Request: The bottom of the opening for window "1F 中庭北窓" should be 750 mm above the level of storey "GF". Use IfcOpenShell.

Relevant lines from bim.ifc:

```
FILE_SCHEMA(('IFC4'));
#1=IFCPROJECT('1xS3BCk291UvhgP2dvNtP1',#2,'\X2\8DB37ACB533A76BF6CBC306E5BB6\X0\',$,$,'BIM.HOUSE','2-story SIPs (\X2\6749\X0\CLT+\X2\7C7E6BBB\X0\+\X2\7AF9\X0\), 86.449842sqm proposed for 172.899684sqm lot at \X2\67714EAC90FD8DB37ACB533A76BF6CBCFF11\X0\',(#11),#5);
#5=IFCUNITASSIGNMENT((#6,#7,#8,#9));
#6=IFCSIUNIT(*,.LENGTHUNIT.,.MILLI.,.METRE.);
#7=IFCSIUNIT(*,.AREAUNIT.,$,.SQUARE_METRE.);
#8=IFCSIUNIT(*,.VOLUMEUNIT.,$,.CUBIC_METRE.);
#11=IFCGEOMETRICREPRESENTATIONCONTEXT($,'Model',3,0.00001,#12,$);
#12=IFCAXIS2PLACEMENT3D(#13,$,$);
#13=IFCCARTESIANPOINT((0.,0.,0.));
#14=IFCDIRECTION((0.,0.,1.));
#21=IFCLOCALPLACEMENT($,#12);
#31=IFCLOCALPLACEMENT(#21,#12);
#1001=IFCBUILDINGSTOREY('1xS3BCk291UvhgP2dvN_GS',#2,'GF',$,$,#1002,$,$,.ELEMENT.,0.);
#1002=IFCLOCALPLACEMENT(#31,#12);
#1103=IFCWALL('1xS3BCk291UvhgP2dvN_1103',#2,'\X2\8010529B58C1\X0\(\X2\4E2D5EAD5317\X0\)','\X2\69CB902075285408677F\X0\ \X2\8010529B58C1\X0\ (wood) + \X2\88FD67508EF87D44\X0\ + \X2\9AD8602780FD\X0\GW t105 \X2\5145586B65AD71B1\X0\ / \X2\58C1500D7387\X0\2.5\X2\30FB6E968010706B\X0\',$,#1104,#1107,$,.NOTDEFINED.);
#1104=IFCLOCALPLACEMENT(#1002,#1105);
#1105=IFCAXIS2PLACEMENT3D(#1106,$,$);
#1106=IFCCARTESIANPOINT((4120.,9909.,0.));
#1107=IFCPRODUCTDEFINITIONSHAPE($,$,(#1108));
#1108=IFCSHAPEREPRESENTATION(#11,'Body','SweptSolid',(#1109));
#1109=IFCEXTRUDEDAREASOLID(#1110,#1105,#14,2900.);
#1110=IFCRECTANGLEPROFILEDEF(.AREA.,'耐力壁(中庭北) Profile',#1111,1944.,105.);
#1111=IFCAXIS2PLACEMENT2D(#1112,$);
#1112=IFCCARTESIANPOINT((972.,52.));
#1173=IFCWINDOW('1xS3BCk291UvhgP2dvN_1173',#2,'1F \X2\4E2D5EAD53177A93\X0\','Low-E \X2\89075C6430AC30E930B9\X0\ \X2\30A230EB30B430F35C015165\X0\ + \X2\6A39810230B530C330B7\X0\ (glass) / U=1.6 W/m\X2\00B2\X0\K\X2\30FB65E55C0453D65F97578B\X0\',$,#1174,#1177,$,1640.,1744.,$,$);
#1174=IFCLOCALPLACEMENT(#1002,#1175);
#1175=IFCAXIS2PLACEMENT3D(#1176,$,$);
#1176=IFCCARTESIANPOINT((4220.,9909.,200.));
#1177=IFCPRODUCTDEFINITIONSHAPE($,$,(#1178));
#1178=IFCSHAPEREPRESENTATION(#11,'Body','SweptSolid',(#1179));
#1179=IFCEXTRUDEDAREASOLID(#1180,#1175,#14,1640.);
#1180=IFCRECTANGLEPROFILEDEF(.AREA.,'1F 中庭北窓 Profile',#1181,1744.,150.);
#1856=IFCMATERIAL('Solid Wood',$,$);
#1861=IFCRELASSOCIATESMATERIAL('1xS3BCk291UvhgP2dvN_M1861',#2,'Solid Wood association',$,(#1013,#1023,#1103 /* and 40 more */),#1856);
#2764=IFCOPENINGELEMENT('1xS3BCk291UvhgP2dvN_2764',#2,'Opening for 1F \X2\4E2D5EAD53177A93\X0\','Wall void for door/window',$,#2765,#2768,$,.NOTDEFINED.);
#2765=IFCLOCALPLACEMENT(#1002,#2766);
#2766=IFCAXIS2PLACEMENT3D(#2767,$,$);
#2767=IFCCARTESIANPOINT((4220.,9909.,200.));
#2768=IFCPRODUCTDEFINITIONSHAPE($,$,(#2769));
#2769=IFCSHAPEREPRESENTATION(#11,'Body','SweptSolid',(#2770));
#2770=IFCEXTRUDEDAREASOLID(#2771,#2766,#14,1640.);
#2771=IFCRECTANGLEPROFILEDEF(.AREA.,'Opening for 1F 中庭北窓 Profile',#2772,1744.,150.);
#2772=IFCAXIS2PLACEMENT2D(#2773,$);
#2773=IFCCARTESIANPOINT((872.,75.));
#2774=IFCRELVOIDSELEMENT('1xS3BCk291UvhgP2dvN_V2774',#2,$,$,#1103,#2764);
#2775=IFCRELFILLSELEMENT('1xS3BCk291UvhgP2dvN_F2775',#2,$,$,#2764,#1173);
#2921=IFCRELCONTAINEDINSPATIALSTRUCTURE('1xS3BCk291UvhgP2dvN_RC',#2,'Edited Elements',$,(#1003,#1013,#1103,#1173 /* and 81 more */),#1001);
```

```python
import numpy as np
import ifcopenshell
import ifcopenshell.api.geometry
import ifcopenshell.geom
import ifcopenshell.util.element
import ifcopenshell.util.placement
import ifcopenshell.util.shape
import ifcopenshell.util.unit

model = ifcopenshell.open("bim.ifc")
unit_scale = ifcopenshell.util.unit.calculate_unit_scale(model)

window = model.by_guid("1xS3BCk291UvhgP2dvN_1173")
opening = window.FillsVoids[0].RelatingOpeningElement
storey = ifcopenshell.util.element.get_container(window, ifc_class="IfcBuildingStorey")
level = ifcopenshell.util.placement.get_local_placement(storey.ObjectPlacement)[2, 3]

# The opening's origin need not be at the sill, so measure its lowest point.
shape = ifcopenshell.geom.create_shape(ifcopenshell.geom.settings(), opening)
bottom = ifcopenshell.util.shape.get_shape_bottom_elevation(shape, shape.geometry) / unit_scale
dz = level + 0.75 / unit_scale - bottom

shift = np.array([0.0, 0.0, dz])
# The window is not placed relative to its opening, so move both.
for product in (opening, window):
    matrix = ifcopenshell.util.placement.get_local_placement(product.ObjectPlacement)
    matrix[:3, 3] += shift
    ifcopenshell.api.geometry.edit_object_placement(model, product=product, matrix=matrix, is_si=False)

print(f"moved by {dz * unit_scale:+.3f} m")

model.write("bim_rev.ifc")
```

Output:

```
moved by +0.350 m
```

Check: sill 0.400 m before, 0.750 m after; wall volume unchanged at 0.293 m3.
